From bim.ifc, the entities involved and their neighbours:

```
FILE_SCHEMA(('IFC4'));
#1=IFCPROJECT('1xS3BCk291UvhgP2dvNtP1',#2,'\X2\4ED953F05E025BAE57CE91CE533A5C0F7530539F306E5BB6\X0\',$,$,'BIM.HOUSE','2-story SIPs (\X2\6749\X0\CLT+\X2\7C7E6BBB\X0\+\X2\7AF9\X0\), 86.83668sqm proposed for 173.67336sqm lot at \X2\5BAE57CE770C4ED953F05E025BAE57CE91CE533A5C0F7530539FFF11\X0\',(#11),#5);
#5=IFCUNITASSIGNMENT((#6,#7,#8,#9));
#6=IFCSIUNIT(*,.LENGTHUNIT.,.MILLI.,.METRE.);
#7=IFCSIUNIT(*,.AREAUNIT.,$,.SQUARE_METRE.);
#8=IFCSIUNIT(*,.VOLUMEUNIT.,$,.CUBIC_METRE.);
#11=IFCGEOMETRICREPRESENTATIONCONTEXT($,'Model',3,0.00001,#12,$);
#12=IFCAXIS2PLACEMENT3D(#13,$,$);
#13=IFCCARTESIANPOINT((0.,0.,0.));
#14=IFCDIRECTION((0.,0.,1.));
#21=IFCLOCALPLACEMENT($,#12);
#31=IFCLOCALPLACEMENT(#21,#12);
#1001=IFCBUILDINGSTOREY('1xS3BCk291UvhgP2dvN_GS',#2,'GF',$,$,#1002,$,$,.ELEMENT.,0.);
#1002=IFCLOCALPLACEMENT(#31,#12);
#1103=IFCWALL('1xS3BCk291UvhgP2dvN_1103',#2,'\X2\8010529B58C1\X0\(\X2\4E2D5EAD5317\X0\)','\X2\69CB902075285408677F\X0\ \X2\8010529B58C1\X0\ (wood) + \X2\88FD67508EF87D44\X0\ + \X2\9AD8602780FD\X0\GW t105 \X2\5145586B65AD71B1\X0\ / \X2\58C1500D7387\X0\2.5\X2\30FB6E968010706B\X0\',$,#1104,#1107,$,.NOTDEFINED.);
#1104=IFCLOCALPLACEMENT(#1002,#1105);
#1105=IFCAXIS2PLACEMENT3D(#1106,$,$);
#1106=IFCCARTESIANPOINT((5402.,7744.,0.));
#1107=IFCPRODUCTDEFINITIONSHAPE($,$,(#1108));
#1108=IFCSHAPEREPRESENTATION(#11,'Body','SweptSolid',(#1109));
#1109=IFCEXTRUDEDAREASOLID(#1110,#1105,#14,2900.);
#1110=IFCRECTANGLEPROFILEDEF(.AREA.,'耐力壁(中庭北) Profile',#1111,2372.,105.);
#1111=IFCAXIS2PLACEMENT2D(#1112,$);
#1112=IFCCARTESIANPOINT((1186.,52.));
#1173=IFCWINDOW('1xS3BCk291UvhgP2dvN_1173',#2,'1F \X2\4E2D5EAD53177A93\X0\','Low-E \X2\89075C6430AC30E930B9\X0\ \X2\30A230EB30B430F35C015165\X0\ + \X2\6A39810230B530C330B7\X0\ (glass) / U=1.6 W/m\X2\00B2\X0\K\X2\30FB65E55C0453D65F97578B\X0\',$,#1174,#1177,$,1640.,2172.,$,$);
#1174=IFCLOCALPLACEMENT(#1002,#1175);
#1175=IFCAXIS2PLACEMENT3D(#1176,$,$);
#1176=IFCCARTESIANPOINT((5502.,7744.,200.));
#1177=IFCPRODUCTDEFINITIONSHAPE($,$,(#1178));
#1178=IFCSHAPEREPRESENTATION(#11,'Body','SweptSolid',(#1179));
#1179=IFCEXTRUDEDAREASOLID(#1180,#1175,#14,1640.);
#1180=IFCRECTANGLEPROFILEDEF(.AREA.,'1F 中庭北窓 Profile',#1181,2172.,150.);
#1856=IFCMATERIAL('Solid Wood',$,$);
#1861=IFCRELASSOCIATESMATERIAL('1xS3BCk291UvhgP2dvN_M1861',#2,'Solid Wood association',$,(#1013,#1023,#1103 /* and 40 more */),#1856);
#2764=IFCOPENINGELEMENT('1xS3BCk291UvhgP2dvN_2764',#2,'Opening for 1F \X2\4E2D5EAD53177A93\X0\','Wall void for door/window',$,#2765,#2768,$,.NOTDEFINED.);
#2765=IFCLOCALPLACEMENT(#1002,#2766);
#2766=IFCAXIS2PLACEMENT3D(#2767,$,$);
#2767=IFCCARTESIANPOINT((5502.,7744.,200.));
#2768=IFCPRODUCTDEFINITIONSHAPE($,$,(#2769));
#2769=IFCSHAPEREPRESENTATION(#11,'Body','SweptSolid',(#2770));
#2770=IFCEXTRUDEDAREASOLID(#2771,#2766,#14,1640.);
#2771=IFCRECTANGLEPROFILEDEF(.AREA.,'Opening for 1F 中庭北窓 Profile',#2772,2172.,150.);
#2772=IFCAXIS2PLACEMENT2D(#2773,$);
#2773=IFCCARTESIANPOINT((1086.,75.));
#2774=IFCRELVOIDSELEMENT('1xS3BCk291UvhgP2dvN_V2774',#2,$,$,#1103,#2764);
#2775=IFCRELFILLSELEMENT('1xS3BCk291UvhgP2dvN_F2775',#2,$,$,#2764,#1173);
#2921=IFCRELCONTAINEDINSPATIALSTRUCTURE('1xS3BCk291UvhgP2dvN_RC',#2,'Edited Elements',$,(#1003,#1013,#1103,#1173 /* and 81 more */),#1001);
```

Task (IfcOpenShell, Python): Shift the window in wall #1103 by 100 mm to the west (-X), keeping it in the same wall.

```python
import ifcopenshell
import ifcopenshell.api.geometry
import ifcopenshell.util.placement
import ifcopenshell.util.unit

model = ifcopenshell.open("bim.ifc")
unit_scale = ifcopenshell.util.unit.calculate_unit_scale(model)

window = model.by_guid("1xS3BCk291UvhgP2dvN_1173")
opening = window.FillsVoids[0].RelatingOpeningElement
wall = opening.VoidsElements[0].RelatingBuildingElement

wall_matrix = ifcopenshell.util.placement.get_local_placement(wall.ObjectPlacement)
shift = wall_matrix[:3, 0] * -0.1 / unit_scale
before = ifcopenshell.util.placement.get_local_placement(window.ObjectPlacement)[:3, 3].copy()

# The window is not placed relative to its opening, so move both.
for product in (opening, window):
    matrix = ifcopenshell.util.placement.get_local_placement(product.ObjectPlacement)
    matrix[:3, 3] += shift
    ifcopenshell.api.geometry.edit_object_placement(model, product=product, matrix=matrix, is_si=False)

after = ifcopenshell.util.placement.get_local_placement(window.ObjectPlacement)[:3, 3]
print("window moved by", (after - before).round(3) + 0.0)

model.write("bim_edited.ifc")
```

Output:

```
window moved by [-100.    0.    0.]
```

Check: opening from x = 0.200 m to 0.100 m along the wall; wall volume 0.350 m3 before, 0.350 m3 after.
